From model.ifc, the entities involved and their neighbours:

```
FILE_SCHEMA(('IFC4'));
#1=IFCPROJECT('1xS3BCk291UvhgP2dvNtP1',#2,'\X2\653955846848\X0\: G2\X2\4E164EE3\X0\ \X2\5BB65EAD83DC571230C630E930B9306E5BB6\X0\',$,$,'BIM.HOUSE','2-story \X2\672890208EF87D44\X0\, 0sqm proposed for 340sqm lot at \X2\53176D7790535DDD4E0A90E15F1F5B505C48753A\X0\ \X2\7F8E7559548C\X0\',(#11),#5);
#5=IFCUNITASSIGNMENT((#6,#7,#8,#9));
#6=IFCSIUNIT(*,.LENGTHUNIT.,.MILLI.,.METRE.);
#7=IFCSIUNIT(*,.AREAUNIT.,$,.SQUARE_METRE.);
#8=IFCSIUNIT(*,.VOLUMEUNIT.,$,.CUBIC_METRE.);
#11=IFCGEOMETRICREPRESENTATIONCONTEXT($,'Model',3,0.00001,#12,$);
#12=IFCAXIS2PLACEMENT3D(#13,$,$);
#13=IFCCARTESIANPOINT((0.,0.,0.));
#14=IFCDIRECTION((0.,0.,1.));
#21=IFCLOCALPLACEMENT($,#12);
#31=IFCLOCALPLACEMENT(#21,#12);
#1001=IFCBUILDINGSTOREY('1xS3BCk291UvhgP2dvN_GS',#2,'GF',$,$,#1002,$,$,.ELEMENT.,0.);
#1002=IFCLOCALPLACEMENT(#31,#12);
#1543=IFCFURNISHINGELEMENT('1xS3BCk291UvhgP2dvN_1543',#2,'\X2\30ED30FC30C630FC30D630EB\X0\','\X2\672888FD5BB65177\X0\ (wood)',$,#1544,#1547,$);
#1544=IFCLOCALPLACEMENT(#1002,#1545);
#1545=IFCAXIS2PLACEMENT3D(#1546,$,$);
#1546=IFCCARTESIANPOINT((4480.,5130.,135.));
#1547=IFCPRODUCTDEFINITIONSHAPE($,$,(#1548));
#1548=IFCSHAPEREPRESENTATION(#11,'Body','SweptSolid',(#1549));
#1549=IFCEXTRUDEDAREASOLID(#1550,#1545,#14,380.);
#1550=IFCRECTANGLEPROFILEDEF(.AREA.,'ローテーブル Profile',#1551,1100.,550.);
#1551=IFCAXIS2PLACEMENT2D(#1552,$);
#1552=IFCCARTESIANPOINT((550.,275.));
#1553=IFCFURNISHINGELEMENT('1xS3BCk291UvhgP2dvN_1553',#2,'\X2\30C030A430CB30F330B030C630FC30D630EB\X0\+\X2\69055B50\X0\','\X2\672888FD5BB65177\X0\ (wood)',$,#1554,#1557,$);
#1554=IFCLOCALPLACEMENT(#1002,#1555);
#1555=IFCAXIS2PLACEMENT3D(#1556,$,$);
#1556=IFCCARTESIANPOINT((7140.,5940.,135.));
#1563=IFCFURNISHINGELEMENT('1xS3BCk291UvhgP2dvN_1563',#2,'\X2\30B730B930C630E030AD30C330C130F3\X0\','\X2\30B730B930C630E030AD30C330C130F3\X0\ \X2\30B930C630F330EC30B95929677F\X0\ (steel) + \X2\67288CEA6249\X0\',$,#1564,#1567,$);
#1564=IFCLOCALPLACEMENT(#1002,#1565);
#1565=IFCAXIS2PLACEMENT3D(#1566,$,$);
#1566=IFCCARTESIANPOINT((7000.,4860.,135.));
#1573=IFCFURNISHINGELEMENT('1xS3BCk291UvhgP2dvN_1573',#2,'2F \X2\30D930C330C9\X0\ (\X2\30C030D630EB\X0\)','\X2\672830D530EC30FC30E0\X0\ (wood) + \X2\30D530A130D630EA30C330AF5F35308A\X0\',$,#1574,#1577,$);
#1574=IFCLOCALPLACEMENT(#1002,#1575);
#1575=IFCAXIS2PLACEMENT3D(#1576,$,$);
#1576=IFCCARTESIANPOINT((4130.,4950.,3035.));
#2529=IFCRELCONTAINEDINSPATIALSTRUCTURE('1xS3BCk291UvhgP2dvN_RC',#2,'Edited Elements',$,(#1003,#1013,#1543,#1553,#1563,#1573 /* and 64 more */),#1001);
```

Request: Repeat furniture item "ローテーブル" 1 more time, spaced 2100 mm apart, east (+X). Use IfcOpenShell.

```python
import numpy as np
import ifcopenshell
import ifcopenshell.api.geometry
import ifcopenshell.api.root
import ifcopenshell.util.element
import ifcopenshell.util.placement
import ifcopenshell.util.unit

model = ifcopenshell.open("model.ifc")
unit_scale = ifcopenshell.util.unit.calculate_unit_scale(model)


def reuse_history(source, copy):
    """copy_class also copies each property set's owner history, people and application; keep the originals."""
    for rel in copy.IsDefinedBy:
        if rel.is_a("IfcRelDefinesByProperties") and (history := rel.RelatingPropertyDefinition.OwnerHistory):
            rel.RelatingPropertyDefinition.OwnerHistory = source.OwnerHistory
            ifcopenshell.util.element.remove_deep2(model, history)


source = model.by_id(1543)
base = ifcopenshell.util.placement.get_local_placement(source.ObjectPlacement)
step = np.array([1.0, 0.0, 0.0]) * 2.1 / unit_scale

for i in range(1, 2):
    copy = ifcopenshell.api.root.copy_class(model, product=source)
    copy.Representation = ifcopenshell.util.element.copy_deep(
        model, source.Representation, exclude=["IfcGeometricRepresentationContext", "IfcRepresentationMap"]
    )
    reuse_history(source, copy)
    matrix = base.copy()
    matrix[:3, 3] += i * step
    print("added at", matrix[:3, 3].round(3) + 0.0)
    ifcopenshell.api.geometry.edit_object_placement(model, product=copy, matrix=matrix, is_si=False)

model.write("model-out.ifc")
```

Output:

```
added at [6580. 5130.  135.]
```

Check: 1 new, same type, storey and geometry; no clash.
